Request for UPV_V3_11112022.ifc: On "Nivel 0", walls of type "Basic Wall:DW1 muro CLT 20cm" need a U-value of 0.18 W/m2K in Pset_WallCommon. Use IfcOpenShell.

First a look at what the model holds.

```python
import ifcopenshell
import ifcopenshell.util.element

model = ifcopenshell.open("UPV_V3_11112022.ifc")
print(model.schema)
storey = next(s for s in model.by_type("IfcBuildingStorey") if s.Name == "Nivel 0")
walls = [e for e in ifcopenshell.util.element.get_decomposition(storey) if e.is_a("IfcWall")]
seen = {}
for e in walls:
    element_type = ifcopenshell.util.element.get_type(e)
    key = (element_type.Name if element_type != e and element_type else None, ifcopenshell.util.element.get_pset(e, "Pset_WallCommon", "ThermalTransmittance"))
    seen[key] = seen.get(key, 0) + 1
for (name, value), count in sorted(seen.items(), key=str):
    print(count, "x", name, "|", value)
```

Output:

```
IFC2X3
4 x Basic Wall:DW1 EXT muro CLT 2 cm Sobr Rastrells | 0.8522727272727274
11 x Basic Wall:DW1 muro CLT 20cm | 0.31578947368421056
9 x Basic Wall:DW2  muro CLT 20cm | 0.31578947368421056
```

```python
import ifcopenshell
import ifcopenshell.api.pset
import ifcopenshell.util.element

model = ifcopenshell.open("UPV_V3_11112022.ifc")

storey = next(s for s in model.by_type("IfcBuildingStorey") if s.Name == "Nivel 0")
walls = [e for e in ifcopenshell.util.element.get_decomposition(storey) if e.is_a("IfcWall")]

count = 0
for e in walls:
    element_type = ifcopenshell.util.element.get_type(e)
    if element_type in (None, e) or element_type.Name != "Basic Wall:DW1 muro CLT 20cm":
        continue
    # add_pset returns the element's existing set when there is one.
    pset = ifcopenshell.api.pset.add_pset(model, product=e, name="Pset_WallCommon")
    ifcopenshell.api.pset.edit_pset(model, pset=pset, properties={"ThermalTransmittance": 0.18})
    count += 1

print(count, "walls updated")

model.write("UPV_V3_11112022_edited.ifc")
```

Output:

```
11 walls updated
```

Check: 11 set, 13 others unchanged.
